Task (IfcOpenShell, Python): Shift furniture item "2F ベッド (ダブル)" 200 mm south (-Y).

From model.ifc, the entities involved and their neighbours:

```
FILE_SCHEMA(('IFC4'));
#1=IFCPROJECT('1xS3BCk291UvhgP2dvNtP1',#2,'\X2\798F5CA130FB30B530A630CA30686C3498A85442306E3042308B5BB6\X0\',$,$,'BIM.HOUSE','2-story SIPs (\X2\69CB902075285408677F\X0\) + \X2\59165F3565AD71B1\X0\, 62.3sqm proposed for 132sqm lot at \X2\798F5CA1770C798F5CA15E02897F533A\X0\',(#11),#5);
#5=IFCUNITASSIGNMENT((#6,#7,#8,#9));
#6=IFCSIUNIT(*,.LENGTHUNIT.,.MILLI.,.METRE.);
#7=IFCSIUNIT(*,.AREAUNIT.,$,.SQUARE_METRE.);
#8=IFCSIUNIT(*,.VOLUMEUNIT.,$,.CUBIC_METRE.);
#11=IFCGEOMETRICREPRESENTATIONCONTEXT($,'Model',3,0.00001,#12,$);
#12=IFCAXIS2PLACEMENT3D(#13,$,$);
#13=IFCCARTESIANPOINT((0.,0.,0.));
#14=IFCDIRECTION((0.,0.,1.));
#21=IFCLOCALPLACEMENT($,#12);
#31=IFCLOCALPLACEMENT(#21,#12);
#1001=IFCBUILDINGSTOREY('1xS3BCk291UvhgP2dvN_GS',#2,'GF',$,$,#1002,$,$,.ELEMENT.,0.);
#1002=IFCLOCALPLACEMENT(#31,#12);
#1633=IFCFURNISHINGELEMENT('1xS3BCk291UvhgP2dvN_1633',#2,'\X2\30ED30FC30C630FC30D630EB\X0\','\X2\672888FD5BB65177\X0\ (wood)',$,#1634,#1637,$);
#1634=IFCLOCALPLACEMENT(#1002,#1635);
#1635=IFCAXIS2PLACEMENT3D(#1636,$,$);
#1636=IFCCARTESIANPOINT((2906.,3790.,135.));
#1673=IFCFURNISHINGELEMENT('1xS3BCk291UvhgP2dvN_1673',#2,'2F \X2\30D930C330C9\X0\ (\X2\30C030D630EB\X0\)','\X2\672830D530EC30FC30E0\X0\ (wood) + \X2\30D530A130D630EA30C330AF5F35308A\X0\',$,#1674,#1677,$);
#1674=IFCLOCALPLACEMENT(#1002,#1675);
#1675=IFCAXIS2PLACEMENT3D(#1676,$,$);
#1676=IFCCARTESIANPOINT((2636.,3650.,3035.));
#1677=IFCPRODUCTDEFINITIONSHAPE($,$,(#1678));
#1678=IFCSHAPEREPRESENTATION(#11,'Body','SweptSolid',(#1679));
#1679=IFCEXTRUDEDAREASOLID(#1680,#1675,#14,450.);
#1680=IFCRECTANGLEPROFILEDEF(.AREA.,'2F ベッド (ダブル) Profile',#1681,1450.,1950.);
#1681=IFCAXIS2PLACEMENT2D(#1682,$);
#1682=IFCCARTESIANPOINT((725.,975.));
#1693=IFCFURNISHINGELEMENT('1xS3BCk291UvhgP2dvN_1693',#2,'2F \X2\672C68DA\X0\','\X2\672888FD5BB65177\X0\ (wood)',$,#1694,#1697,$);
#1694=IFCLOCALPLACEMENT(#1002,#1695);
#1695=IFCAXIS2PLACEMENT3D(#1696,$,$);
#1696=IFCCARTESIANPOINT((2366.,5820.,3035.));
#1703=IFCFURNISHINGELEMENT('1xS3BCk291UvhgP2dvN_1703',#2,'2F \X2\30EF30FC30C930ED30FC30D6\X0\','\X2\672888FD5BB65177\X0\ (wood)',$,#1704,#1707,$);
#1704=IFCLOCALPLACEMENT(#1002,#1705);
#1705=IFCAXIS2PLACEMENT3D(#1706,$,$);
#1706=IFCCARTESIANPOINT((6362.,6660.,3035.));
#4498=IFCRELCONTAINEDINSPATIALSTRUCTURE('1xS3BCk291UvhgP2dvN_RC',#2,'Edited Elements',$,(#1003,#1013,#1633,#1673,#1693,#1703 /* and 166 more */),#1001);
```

```python
import ifcopenshell
import ifcopenshell.api.geometry
import ifcopenshell.util.placement
import ifcopenshell.util.unit

model = ifcopenshell.open("model.ifc")
unit_scale = ifcopenshell.util.unit.calculate_unit_scale(model)

item = model.by_guid("1xS3BCk291UvhgP2dvN_1673")
matrix = ifcopenshell.util.placement.get_local_placement(item.ObjectPlacement)
matrix[1, 3] -= 0.2 / unit_scale
ifcopenshell.api.geometry.edit_object_placement(model, product=item, matrix=matrix, is_si=False)

print(ifcopenshell.util.placement.get_local_placement(item.ObjectPlacement).round(3) + 0.0)

model.write("model_v2.ifc")
```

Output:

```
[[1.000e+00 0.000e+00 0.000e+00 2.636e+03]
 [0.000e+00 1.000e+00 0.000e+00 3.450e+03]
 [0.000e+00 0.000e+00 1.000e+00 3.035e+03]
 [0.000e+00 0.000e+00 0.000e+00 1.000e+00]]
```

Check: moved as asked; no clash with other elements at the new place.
